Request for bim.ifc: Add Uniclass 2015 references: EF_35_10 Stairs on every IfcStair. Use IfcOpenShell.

First a look at what the model holds.

```python
import ifcopenshell

model = ifcopenshell.open("bim.ifc")
print(model.schema)
print("classifications:", [c.Name for c in model.by_type("IfcClassification")])
for ifc_class in ("IfcDoor", "IfcRoof", "IfcStair", "IfcWall", "IfcWindow"):
    print(ifc_class, len(model.by_type(ifc_class)))
```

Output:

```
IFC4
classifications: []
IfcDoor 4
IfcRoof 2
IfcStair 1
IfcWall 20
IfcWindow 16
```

```python
import ifcopenshell
import ifcopenshell.api.classification

model = ifcopenshell.open("bim.ifc")

system = ifcopenshell.api.classification.add_classification(model, classification="Uniclass 2015")

codes = {
    "IfcStair": ("EF_35_10", "Stairs"),
}
for ifc_class, (code, name) in codes.items():
    products = model.by_type(ifc_class)
    ifcopenshell.api.classification.add_reference(
        model, products=products, classification=system, identification=code, name=name
    )
    print(code, len(products))

model.write("bim_v2.ifc")
```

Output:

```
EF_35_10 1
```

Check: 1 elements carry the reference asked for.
